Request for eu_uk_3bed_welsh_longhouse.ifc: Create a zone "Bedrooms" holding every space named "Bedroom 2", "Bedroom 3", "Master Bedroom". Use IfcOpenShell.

First a look at what the model holds.

```python
import ifcopenshell

model = ifcopenshell.open("eu_uk_3bed_welsh_longhouse.ifc")
print(model.schema)
seen = {}
for space in model.by_type("IfcSpace"):
    seen[space.LongName] = seen.get(space.LongName, 0) + 1
for name, count in sorted(seen.items(), key=str):
    print(count, "x", name)
print("zones:", [z.Name for z in model.by_type("IfcZone")][:20])
```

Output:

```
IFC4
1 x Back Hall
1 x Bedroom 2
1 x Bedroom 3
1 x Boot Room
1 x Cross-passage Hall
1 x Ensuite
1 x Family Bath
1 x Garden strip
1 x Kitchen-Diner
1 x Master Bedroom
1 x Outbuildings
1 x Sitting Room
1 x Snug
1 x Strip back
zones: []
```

```python
import ifcopenshell
import ifcopenshell.api.group
import ifcopenshell.api.root

model = ifcopenshell.open("eu_uk_3bed_welsh_longhouse.ifc")

names = {"Bedroom 2", "Bedroom 3", "Master Bedroom"}
spaces = [s for s in model.by_type("IfcSpace") if s.LongName in names]

zone = ifcopenshell.api.root.create_entity(model, ifc_class="IfcZone", name="Bedrooms")
ifcopenshell.api.group.assign_group(model, products=spaces, group=zone)
print(len(spaces), "spaces in", zone.Name)

model.write("eu_uk_3bed_welsh_longhouse_updated.ifc")
```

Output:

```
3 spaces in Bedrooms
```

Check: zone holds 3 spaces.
